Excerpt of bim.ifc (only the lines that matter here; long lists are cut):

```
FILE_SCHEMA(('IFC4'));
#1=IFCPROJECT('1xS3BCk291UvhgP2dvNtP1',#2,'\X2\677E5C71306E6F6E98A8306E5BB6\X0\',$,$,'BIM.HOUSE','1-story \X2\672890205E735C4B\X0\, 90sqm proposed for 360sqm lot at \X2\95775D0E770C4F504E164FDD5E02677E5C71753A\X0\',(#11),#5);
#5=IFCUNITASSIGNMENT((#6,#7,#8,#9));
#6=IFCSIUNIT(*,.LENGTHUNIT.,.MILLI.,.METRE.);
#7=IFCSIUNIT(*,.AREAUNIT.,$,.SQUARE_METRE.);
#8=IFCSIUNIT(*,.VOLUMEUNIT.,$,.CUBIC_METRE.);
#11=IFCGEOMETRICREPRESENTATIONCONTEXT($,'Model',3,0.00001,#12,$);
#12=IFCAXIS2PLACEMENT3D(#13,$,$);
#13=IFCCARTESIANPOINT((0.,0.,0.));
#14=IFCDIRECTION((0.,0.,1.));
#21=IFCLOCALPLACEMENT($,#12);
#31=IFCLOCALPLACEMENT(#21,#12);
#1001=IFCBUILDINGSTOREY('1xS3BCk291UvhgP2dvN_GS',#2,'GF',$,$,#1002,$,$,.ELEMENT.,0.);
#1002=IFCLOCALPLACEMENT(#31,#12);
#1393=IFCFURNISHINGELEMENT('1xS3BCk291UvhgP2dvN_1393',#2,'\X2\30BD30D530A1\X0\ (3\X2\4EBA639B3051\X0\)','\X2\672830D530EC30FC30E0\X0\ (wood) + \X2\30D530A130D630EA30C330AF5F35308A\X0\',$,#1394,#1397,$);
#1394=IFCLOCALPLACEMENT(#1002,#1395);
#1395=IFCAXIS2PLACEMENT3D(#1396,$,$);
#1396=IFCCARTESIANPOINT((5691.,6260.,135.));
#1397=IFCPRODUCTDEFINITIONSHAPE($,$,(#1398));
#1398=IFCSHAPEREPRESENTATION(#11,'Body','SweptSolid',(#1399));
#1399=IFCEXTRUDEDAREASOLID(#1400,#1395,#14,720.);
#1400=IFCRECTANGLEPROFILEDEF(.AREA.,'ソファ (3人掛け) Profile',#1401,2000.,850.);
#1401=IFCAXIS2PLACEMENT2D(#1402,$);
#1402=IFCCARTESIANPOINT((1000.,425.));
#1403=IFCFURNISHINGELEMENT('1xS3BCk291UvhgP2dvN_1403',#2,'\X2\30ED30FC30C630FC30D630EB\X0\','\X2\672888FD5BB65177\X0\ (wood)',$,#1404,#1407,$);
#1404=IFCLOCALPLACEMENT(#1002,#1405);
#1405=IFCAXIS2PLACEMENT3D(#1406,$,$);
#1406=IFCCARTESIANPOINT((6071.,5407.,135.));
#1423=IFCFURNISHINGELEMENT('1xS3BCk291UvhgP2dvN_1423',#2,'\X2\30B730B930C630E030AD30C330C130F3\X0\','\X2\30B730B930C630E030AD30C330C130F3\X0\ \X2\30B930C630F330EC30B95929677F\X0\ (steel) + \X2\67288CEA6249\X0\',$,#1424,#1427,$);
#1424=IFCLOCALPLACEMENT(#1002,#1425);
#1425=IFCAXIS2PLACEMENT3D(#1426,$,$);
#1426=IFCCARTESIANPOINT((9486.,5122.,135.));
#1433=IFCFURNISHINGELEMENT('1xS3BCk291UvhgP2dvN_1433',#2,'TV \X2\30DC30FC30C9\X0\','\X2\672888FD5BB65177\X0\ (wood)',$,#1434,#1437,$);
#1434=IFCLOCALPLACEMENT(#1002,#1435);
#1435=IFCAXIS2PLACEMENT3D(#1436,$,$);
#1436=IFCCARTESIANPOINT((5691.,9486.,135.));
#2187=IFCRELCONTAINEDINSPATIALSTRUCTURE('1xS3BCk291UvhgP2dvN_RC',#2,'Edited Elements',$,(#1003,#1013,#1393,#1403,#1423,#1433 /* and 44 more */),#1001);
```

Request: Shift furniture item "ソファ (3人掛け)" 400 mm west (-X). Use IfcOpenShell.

```python
import ifcopenshell
import ifcopenshell.api.geometry
import ifcopenshell.util.placement
import ifcopenshell.util.unit

model = ifcopenshell.open("bim.ifc")
unit_scale = ifcopenshell.util.unit.calculate_unit_scale(model)

item = model.by_id(1393)
matrix = ifcopenshell.util.placement.get_local_placement(item.ObjectPlacement)
matrix[0, 3] -= 0.4 / unit_scale
ifcopenshell.api.geometry.edit_object_placement(model, product=item, matrix=matrix, is_si=False)

print(ifcopenshell.util.placement.get_local_placement(item.ObjectPlacement).round(3) + 0.0)

model.write("bim_rev.ifc")
```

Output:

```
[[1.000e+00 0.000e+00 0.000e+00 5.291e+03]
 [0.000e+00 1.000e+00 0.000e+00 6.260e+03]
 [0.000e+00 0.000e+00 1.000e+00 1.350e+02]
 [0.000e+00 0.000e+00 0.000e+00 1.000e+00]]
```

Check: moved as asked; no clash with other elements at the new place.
